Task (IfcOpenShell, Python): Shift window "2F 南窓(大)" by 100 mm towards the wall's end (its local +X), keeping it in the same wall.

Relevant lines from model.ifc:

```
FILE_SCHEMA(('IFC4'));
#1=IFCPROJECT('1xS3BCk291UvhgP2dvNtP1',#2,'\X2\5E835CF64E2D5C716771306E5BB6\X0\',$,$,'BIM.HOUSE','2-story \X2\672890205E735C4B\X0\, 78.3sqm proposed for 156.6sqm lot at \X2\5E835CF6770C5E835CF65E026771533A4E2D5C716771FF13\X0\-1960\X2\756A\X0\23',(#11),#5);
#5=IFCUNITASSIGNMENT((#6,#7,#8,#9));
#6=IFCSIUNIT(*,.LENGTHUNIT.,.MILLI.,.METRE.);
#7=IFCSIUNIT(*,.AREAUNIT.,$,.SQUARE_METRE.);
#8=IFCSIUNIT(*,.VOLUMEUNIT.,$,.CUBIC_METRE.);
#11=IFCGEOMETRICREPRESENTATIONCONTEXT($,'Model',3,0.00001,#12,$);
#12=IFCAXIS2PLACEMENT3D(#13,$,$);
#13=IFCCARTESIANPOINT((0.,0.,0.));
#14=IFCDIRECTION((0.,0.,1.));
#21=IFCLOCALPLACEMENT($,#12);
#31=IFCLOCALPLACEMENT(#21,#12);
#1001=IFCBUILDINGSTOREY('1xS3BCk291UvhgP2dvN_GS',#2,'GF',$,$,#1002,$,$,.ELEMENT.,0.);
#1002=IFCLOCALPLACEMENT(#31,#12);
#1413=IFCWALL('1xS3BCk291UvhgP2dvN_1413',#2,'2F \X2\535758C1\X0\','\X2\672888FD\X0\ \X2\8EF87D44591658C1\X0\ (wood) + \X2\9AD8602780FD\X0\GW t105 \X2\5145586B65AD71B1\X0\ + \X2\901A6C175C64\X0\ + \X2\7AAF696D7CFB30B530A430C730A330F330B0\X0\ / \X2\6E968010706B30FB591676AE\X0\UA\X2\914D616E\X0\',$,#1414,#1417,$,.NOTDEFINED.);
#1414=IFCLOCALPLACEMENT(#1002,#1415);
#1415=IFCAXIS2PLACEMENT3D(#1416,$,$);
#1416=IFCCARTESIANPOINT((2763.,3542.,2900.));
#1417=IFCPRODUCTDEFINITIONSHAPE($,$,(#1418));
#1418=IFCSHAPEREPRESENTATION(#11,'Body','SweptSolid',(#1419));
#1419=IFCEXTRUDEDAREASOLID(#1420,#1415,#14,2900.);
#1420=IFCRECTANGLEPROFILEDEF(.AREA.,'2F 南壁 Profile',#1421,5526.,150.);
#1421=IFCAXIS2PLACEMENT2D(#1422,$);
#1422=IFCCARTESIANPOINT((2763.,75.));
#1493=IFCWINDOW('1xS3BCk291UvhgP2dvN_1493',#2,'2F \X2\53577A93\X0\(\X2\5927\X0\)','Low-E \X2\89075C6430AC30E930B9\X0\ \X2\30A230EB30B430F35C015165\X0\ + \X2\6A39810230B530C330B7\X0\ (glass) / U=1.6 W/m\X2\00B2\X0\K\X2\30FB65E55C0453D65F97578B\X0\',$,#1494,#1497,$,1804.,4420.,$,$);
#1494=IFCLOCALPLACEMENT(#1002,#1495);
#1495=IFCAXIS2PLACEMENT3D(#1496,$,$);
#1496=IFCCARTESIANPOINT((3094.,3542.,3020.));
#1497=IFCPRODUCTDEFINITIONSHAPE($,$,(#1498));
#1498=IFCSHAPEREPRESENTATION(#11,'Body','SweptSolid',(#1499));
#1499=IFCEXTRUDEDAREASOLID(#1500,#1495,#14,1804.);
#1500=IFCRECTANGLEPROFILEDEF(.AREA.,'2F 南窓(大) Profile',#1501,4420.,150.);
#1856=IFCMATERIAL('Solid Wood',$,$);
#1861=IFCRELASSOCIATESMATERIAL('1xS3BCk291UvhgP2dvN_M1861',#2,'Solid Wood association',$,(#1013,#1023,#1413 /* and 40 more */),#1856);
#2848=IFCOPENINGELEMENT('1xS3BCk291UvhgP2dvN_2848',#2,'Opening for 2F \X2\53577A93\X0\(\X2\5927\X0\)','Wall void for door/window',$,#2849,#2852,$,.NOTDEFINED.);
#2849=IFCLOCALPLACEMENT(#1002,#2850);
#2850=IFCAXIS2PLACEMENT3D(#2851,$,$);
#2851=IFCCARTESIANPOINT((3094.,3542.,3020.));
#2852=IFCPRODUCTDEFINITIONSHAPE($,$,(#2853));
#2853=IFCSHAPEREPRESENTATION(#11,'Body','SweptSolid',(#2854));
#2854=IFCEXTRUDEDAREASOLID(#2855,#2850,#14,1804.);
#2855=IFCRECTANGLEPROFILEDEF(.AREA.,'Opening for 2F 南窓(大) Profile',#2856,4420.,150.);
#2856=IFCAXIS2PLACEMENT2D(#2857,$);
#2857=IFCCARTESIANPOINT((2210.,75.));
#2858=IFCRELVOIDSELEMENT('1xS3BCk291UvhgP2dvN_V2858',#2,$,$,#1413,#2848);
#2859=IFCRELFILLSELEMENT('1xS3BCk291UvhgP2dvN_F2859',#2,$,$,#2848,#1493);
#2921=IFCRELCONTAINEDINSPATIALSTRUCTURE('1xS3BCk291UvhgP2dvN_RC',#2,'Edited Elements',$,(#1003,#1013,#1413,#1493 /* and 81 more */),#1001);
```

```python
import ifcopenshell
import ifcopenshell.api.geometry
import ifcopenshell.util.placement

model = ifcopenshell.open("model.ifc")

window = model.by_id(1493)
opening = window.FillsVoids[0].RelatingOpeningElement
wall = opening.VoidsElements[0].RelatingBuildingElement

wall_matrix = ifcopenshell.util.placement.get_local_placement(wall.ObjectPlacement)
shift = wall_matrix[:3, 0] * 100.0
before = ifcopenshell.util.placement.get_local_placement(window.ObjectPlacement)[:3, 3].copy()

# The window is not placed relative to its opening, so move both.
for product in (opening, window):
    matrix = ifcopenshell.util.placement.get_local_placement(product.ObjectPlacement)
    matrix[:3, 3] += shift
    ifcopenshell.api.geometry.edit_object_placement(model, product=product, matrix=matrix, is_si=False)

after = ifcopenshell.util.placement.get_local_placement(window.ObjectPlacement)[:3, 3]
print("window moved by", (after - before).round(3) + 0.0)

model.write("model_updated.ifc")
```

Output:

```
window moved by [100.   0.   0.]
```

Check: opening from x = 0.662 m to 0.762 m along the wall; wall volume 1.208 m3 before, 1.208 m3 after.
